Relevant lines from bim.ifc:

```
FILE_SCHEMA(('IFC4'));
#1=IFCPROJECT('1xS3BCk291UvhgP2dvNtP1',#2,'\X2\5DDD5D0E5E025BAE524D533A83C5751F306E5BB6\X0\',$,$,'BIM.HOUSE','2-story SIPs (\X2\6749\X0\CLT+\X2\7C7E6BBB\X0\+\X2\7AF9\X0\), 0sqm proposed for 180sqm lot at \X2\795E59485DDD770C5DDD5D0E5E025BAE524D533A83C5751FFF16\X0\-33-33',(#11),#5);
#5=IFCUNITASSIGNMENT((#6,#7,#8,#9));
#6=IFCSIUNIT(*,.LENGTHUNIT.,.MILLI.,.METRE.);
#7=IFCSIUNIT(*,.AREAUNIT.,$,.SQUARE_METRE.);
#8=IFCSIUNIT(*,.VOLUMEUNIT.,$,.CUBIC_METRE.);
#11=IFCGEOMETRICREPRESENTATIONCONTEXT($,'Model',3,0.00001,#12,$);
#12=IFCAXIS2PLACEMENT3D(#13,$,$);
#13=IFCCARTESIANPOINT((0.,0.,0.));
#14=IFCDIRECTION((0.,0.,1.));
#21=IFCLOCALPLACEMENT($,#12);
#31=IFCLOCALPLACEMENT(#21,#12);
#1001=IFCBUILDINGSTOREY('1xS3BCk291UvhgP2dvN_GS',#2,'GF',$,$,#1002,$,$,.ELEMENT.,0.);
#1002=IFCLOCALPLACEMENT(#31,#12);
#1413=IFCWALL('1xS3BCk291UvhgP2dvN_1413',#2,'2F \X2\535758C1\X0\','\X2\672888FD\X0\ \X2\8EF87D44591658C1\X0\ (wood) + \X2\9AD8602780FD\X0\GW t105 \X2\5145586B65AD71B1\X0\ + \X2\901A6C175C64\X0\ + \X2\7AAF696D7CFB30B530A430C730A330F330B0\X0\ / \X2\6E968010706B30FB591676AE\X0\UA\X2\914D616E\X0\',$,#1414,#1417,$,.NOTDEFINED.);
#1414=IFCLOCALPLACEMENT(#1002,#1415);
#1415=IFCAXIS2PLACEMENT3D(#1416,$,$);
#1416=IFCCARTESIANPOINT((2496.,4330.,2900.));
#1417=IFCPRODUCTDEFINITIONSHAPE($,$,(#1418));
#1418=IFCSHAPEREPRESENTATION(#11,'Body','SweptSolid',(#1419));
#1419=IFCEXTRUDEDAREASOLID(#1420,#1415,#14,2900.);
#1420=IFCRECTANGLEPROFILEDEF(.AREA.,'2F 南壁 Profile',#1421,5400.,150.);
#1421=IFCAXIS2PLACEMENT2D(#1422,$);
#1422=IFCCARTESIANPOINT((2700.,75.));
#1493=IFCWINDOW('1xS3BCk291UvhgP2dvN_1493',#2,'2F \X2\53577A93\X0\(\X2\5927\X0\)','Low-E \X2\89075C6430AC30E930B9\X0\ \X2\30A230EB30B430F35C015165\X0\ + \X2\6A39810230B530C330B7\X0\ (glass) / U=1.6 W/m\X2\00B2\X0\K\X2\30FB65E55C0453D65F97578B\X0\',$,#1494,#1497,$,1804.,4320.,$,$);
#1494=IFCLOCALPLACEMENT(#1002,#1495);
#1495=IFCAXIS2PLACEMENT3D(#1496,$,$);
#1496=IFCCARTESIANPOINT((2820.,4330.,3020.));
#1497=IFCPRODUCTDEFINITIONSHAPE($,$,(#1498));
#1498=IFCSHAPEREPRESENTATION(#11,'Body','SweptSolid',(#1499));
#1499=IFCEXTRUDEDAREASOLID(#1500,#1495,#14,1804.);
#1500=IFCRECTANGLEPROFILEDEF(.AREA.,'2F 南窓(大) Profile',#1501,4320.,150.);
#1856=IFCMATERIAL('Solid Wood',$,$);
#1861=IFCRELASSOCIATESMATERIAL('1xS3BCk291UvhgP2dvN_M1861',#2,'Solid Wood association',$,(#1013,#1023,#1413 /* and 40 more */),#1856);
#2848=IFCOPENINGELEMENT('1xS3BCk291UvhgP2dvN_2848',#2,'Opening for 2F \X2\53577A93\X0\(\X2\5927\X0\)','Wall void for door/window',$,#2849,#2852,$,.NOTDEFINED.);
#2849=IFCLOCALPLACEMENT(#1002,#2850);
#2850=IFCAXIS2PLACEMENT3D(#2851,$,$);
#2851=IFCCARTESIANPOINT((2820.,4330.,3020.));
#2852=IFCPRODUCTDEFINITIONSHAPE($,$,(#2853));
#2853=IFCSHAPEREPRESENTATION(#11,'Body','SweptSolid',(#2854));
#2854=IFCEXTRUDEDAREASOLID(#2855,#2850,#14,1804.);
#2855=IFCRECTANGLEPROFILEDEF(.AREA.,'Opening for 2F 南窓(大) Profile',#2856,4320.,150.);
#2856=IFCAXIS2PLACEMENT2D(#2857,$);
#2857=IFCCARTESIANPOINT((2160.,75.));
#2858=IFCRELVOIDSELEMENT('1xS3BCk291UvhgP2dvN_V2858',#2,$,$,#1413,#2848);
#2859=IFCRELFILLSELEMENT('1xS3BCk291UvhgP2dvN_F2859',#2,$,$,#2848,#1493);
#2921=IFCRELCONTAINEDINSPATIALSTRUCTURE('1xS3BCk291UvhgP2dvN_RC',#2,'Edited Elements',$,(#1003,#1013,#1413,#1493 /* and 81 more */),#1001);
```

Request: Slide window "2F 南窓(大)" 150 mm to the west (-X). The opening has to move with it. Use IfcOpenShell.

```python
import ifcopenshell
import ifcopenshell.api.geometry
import ifcopenshell.util.placement

model = ifcopenshell.open("bim.ifc")

window = model.by_guid("1xS3BCk291UvhgP2dvN_1493")
opening = window.FillsVoids[0].RelatingOpeningElement
wall = opening.VoidsElements[0].RelatingBuildingElement

wall_matrix = ifcopenshell.util.placement.get_local_placement(wall.ObjectPlacement)
shift = wall_matrix[:3, 0] * -150.0
before = ifcopenshell.util.placement.get_local_placement(window.ObjectPlacement)[:3, 3].copy()

# The window is not placed relative to its opening, so move both.
for product in (opening, window):
    matrix = ifcopenshell.util.placement.get_local_placement(product.ObjectPlacement)
    matrix[:3, 3] += shift
    ifcopenshell.api.geometry.edit_object_placement(model, product=product, matrix=matrix, is_si=False)

after = ifcopenshell.util.placement.get_local_placement(window.ObjectPlacement)[:3, 3]
print("window moved by", (after - before).round(3) + 0.0)

model.write("bim_v2.ifc")
```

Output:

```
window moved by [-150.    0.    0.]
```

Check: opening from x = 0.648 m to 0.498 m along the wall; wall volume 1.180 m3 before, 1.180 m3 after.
